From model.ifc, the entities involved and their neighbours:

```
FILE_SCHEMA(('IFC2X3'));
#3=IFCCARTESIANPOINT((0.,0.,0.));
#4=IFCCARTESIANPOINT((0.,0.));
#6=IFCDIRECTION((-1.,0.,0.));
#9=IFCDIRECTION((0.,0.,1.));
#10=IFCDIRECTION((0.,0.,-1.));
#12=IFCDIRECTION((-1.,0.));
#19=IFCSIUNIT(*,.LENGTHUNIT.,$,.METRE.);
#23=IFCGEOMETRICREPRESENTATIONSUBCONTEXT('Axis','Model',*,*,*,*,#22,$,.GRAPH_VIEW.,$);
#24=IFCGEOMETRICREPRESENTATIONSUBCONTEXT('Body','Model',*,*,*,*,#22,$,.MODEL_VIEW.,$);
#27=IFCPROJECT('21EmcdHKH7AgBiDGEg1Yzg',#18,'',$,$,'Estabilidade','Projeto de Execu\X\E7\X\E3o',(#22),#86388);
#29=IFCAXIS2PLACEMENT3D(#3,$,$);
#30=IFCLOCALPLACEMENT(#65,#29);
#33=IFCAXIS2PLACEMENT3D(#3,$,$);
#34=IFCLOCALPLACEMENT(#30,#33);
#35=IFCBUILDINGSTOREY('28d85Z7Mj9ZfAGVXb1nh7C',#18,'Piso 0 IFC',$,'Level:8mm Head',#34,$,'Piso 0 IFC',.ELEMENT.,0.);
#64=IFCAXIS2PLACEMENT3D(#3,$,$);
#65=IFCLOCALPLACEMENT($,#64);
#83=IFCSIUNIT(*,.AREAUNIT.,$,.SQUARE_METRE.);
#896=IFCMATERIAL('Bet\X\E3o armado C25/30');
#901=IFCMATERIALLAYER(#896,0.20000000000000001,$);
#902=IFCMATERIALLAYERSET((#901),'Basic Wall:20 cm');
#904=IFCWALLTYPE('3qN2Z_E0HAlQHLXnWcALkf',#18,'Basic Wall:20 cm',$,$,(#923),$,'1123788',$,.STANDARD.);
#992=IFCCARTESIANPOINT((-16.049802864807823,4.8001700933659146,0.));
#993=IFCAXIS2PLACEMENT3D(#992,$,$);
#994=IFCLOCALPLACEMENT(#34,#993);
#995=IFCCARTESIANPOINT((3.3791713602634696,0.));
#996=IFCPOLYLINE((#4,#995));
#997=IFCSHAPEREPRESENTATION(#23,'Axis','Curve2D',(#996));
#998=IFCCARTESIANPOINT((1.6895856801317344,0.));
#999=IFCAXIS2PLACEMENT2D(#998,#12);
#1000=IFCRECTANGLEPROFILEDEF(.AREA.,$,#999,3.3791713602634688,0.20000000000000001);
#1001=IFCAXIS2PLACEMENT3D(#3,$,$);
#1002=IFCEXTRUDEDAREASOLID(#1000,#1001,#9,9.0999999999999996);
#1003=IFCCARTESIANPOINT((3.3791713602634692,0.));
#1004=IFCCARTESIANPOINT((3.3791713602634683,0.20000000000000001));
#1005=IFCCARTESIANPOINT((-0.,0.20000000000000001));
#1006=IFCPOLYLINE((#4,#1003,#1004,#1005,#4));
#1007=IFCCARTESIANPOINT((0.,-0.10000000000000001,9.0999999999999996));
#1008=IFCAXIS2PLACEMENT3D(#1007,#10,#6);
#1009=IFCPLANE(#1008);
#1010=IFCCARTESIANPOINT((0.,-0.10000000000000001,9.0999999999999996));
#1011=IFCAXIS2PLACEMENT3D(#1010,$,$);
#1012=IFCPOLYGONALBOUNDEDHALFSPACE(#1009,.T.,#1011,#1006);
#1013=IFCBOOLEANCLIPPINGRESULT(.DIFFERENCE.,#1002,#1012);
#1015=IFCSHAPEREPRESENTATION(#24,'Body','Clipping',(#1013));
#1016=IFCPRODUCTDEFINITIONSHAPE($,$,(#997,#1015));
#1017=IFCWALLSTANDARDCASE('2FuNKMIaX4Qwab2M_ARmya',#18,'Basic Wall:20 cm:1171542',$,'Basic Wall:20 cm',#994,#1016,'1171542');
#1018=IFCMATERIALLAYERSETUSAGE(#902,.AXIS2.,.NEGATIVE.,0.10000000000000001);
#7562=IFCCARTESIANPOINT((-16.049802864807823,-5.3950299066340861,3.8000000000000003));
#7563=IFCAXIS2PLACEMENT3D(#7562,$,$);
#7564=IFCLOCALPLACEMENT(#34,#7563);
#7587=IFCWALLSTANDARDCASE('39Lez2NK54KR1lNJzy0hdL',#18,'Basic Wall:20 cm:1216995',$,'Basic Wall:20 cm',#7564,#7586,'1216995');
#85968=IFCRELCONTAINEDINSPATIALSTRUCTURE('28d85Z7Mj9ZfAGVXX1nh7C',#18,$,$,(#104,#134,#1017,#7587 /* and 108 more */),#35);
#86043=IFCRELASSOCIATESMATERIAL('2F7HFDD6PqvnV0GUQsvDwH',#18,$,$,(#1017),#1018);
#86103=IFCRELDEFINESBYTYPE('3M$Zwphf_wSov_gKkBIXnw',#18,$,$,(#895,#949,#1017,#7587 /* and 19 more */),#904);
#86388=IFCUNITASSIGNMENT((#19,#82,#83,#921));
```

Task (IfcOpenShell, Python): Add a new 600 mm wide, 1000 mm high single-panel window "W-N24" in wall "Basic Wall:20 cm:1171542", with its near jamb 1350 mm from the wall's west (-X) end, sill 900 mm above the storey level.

```python
import numpy as np
import ifcopenshell
import ifcopenshell.api.feature
import ifcopenshell.api.geometry
import ifcopenshell.api.root
import ifcopenshell.api.spatial
import ifcopenshell.api.type
import ifcopenshell.geom
import ifcopenshell.util.element
import ifcopenshell.util.placement
import ifcopenshell.util.representation
import ifcopenshell.util.shape
import ifcopenshell.util.unit

model = ifcopenshell.open("model.ifc")
unit_scale = ifcopenshell.util.unit.calculate_unit_scale(model)
settings = ifcopenshell.geom.settings()


def volume(element):
    """Net volume in cubic metres, openings subtracted."""
    shape = ifcopenshell.geom.create_shape(settings, element)
    return ifcopenshell.util.shape.get_volume(shape.geometry)


wall = model.by_guid("2FuNKMIaX4Qwab2M_ARmya")
storey = ifcopenshell.util.element.get_container(wall, ifc_class="IfcBuildingStorey")
context = ifcopenshell.util.representation.get_context(model, "Model", "Body", "MODEL_VIEW")
before = volume(wall)

width, height, from_end, sill = 0.6, 1, 1.35, 0.9  # metres

# The wall runs along its own X axis, and the end named is its -X end.
wall_shape = ifcopenshell.geom.create_shape(settings, wall)
x, y, z = ifcopenshell.util.shape.get_vertices(wall_shape.geometry).T
start = x.min() + from_end
face, thickness = float(y.min()), float(y.max() - y.min())
wall_matrix = ifcopenshell.util.placement.get_local_placement(wall.ObjectPlacement)
level = ifcopenshell.util.placement.get_local_placement(storey.ObjectPlacement)[2, 3]


def in_wall(x, y):
    """Placement at x, y metres in the wall's axes, at sill height."""
    matrix = wall_matrix.copy()
    matrix[:, 3] = wall_matrix @ np.array([x / unit_scale, y / unit_scale, 0.0, 1.0])
    matrix[2, 3] = level + sill / unit_scale
    return matrix


# Opening: a box that overshoots both wall faces by 50 mm.
opening = ifcopenshell.api.root.create_entity(model, ifc_class="IfcOpeningElement")
box = ifcopenshell.api.geometry.add_wall_representation(
    model, context=context, length=width, height=height, thickness=thickness + 0.1
)
ifcopenshell.api.geometry.assign_representation(model, product=opening, representation=box)
ifcopenshell.api.geometry.edit_object_placement(model, product=opening, matrix=in_wall(start, face - 0.05), is_si=False)
ifcopenshell.api.feature.add_feature(model, feature=opening, element=wall)

window = ifcopenshell.api.root.create_entity(model, ifc_class="IfcWindow", name="W-N24")
window.OverallWidth, window.OverallHeight = width / unit_scale, height / unit_scale
body = ifcopenshell.api.geometry.add_window_representation(
    model,
    context=context,
    overall_width=window.OverallWidth,
    overall_height=window.OverallHeight,
    partition_type="SINGLE_PANEL",
)
ifcopenshell.api.geometry.assign_representation(model, product=window, representation=body)
ifcopenshell.api.spatial.assign_container(model, products=[window], relating_structure=storey)
fills = ifcopenshell.api.feature.add_filling(model, opening=opening, element=window)
fills.OwnerHistory = window.OwnerHistory  # required in IFC2X3

# IFC2X3 keeps the operation on the window style.
style = ifcopenshell.api.root.create_entity(model, ifc_class="IfcWindowStyle", name="W-N24")
style.OperationType, style.ConstructionType = "SINGLE_PANEL", "NOTDEFINED"
style.ParameterTakesPrecedence = style.Sizeable = False
ifcopenshell.api.type.assign_type(model, related_objects=[window], relating_type=style)

# Centre the window in the wall's thickness.
ifcopenshell.api.geometry.edit_object_placement(model, product=window, matrix=in_wall(start, face), is_si=False)
window_shape = ifcopenshell.geom.create_shape(settings, window)
depth = ifcopenshell.util.shape.get_vertices(window_shape.geometry)[:, 1]
offset = face + thickness / 2 - (depth.min() + depth.max()) / 2
ifcopenshell.api.geometry.edit_object_placement(model, product=window, matrix=in_wall(start, offset), is_si=False)

after = volume(wall)

print(f"wall volume {before:.3f} -> {after:.3f} m3")

model.write("model_edited.ifc")
```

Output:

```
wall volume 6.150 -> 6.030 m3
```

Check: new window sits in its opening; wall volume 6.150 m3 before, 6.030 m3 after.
